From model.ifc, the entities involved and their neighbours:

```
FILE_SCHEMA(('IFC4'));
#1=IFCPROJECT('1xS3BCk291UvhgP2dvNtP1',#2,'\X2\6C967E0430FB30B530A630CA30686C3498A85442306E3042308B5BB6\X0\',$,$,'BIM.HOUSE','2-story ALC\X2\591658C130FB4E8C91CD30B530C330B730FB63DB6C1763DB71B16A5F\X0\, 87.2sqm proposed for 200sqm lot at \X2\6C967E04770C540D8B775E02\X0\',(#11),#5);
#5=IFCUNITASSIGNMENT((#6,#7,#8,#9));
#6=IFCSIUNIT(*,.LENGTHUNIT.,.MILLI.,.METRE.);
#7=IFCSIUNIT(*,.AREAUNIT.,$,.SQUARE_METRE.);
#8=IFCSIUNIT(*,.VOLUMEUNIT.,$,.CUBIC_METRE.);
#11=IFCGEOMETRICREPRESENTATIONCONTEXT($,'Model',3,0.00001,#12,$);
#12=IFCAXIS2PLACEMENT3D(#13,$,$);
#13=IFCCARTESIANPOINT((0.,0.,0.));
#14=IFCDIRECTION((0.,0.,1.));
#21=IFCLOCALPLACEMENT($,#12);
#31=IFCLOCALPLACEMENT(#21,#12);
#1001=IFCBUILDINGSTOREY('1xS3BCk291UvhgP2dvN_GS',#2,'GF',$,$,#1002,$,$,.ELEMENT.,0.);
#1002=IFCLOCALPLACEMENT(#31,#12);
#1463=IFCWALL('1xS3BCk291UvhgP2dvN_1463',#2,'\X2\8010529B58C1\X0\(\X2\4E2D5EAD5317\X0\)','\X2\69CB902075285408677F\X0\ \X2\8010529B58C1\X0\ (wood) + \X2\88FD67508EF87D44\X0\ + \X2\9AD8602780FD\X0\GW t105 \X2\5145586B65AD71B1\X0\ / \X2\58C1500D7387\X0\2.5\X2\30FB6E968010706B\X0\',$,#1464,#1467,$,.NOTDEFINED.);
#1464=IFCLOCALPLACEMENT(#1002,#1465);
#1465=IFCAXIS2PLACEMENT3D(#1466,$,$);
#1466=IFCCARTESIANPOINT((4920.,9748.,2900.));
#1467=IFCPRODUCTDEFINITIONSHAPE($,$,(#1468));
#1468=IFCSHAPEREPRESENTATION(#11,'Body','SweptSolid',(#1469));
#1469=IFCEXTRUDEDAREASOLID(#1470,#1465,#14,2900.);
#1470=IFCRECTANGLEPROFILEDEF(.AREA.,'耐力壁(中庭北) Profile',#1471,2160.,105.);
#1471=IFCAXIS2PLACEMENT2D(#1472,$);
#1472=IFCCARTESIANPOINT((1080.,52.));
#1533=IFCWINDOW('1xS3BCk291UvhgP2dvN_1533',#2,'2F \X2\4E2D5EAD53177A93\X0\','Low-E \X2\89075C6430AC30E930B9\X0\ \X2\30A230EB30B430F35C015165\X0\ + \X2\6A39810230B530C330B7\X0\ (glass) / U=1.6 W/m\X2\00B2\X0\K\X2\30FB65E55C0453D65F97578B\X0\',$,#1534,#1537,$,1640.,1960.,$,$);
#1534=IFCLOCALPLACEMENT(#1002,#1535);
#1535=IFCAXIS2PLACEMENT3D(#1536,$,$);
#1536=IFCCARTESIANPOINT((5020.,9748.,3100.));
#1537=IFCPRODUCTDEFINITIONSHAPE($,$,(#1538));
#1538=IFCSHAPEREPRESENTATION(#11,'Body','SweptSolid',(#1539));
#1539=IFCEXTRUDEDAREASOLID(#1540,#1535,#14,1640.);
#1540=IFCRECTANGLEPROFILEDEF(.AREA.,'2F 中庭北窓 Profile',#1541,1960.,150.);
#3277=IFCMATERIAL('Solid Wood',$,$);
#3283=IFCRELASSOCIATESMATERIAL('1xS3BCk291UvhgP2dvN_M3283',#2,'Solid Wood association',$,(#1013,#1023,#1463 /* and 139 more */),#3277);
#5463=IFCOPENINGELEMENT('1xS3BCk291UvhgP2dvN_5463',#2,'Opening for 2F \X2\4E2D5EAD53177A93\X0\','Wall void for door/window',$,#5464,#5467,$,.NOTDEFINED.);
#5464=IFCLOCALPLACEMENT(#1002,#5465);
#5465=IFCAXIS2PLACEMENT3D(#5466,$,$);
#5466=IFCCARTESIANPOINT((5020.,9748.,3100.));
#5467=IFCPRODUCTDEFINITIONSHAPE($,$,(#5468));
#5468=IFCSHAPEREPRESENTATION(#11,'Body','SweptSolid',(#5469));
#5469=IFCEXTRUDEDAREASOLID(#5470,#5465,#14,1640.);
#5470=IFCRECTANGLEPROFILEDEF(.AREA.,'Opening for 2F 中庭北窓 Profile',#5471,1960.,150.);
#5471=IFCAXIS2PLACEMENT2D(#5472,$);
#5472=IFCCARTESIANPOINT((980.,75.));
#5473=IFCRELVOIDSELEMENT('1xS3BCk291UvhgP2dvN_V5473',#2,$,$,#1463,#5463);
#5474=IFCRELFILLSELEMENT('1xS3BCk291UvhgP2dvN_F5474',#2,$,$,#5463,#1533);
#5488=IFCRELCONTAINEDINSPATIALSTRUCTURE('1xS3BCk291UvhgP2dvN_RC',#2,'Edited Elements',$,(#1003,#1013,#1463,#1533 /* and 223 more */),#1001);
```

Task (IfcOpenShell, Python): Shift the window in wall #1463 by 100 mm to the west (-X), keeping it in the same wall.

```python
import ifcopenshell
import ifcopenshell.api.geometry
import ifcopenshell.util.placement
import ifcopenshell.util.unit

model = ifcopenshell.open("model.ifc")
unit_scale = ifcopenshell.util.unit.calculate_unit_scale(model)

window = model.by_guid("1xS3BCk291UvhgP2dvN_1533")
opening = window.FillsVoids[0].RelatingOpeningElement
wall = opening.VoidsElements[0].RelatingBuildingElement

wall_matrix = ifcopenshell.util.placement.get_local_placement(wall.ObjectPlacement)
shift = wall_matrix[:3, 0] * -0.1 / unit_scale
before = ifcopenshell.util.placement.get_local_placement(window.ObjectPlacement)[:3, 3].copy()

# The window is not placed relative to its opening, so move both.
for product in (opening, window):
    matrix = ifcopenshell.util.placement.get_local_placement(product.ObjectPlacement)
    matrix[:3, 3] += shift
    ifcopenshell.api.geometry.edit_object_placement(model, product=product, matrix=matrix, is_si=False)

after = ifcopenshell.util.placement.get_local_placement(window.ObjectPlacement)[:3, 3]
print("window moved by", (after - before).round(3) + 0.0)

model.write("model_edited.ifc")
```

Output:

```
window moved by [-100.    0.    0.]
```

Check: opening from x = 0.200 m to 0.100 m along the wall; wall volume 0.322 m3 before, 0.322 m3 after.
